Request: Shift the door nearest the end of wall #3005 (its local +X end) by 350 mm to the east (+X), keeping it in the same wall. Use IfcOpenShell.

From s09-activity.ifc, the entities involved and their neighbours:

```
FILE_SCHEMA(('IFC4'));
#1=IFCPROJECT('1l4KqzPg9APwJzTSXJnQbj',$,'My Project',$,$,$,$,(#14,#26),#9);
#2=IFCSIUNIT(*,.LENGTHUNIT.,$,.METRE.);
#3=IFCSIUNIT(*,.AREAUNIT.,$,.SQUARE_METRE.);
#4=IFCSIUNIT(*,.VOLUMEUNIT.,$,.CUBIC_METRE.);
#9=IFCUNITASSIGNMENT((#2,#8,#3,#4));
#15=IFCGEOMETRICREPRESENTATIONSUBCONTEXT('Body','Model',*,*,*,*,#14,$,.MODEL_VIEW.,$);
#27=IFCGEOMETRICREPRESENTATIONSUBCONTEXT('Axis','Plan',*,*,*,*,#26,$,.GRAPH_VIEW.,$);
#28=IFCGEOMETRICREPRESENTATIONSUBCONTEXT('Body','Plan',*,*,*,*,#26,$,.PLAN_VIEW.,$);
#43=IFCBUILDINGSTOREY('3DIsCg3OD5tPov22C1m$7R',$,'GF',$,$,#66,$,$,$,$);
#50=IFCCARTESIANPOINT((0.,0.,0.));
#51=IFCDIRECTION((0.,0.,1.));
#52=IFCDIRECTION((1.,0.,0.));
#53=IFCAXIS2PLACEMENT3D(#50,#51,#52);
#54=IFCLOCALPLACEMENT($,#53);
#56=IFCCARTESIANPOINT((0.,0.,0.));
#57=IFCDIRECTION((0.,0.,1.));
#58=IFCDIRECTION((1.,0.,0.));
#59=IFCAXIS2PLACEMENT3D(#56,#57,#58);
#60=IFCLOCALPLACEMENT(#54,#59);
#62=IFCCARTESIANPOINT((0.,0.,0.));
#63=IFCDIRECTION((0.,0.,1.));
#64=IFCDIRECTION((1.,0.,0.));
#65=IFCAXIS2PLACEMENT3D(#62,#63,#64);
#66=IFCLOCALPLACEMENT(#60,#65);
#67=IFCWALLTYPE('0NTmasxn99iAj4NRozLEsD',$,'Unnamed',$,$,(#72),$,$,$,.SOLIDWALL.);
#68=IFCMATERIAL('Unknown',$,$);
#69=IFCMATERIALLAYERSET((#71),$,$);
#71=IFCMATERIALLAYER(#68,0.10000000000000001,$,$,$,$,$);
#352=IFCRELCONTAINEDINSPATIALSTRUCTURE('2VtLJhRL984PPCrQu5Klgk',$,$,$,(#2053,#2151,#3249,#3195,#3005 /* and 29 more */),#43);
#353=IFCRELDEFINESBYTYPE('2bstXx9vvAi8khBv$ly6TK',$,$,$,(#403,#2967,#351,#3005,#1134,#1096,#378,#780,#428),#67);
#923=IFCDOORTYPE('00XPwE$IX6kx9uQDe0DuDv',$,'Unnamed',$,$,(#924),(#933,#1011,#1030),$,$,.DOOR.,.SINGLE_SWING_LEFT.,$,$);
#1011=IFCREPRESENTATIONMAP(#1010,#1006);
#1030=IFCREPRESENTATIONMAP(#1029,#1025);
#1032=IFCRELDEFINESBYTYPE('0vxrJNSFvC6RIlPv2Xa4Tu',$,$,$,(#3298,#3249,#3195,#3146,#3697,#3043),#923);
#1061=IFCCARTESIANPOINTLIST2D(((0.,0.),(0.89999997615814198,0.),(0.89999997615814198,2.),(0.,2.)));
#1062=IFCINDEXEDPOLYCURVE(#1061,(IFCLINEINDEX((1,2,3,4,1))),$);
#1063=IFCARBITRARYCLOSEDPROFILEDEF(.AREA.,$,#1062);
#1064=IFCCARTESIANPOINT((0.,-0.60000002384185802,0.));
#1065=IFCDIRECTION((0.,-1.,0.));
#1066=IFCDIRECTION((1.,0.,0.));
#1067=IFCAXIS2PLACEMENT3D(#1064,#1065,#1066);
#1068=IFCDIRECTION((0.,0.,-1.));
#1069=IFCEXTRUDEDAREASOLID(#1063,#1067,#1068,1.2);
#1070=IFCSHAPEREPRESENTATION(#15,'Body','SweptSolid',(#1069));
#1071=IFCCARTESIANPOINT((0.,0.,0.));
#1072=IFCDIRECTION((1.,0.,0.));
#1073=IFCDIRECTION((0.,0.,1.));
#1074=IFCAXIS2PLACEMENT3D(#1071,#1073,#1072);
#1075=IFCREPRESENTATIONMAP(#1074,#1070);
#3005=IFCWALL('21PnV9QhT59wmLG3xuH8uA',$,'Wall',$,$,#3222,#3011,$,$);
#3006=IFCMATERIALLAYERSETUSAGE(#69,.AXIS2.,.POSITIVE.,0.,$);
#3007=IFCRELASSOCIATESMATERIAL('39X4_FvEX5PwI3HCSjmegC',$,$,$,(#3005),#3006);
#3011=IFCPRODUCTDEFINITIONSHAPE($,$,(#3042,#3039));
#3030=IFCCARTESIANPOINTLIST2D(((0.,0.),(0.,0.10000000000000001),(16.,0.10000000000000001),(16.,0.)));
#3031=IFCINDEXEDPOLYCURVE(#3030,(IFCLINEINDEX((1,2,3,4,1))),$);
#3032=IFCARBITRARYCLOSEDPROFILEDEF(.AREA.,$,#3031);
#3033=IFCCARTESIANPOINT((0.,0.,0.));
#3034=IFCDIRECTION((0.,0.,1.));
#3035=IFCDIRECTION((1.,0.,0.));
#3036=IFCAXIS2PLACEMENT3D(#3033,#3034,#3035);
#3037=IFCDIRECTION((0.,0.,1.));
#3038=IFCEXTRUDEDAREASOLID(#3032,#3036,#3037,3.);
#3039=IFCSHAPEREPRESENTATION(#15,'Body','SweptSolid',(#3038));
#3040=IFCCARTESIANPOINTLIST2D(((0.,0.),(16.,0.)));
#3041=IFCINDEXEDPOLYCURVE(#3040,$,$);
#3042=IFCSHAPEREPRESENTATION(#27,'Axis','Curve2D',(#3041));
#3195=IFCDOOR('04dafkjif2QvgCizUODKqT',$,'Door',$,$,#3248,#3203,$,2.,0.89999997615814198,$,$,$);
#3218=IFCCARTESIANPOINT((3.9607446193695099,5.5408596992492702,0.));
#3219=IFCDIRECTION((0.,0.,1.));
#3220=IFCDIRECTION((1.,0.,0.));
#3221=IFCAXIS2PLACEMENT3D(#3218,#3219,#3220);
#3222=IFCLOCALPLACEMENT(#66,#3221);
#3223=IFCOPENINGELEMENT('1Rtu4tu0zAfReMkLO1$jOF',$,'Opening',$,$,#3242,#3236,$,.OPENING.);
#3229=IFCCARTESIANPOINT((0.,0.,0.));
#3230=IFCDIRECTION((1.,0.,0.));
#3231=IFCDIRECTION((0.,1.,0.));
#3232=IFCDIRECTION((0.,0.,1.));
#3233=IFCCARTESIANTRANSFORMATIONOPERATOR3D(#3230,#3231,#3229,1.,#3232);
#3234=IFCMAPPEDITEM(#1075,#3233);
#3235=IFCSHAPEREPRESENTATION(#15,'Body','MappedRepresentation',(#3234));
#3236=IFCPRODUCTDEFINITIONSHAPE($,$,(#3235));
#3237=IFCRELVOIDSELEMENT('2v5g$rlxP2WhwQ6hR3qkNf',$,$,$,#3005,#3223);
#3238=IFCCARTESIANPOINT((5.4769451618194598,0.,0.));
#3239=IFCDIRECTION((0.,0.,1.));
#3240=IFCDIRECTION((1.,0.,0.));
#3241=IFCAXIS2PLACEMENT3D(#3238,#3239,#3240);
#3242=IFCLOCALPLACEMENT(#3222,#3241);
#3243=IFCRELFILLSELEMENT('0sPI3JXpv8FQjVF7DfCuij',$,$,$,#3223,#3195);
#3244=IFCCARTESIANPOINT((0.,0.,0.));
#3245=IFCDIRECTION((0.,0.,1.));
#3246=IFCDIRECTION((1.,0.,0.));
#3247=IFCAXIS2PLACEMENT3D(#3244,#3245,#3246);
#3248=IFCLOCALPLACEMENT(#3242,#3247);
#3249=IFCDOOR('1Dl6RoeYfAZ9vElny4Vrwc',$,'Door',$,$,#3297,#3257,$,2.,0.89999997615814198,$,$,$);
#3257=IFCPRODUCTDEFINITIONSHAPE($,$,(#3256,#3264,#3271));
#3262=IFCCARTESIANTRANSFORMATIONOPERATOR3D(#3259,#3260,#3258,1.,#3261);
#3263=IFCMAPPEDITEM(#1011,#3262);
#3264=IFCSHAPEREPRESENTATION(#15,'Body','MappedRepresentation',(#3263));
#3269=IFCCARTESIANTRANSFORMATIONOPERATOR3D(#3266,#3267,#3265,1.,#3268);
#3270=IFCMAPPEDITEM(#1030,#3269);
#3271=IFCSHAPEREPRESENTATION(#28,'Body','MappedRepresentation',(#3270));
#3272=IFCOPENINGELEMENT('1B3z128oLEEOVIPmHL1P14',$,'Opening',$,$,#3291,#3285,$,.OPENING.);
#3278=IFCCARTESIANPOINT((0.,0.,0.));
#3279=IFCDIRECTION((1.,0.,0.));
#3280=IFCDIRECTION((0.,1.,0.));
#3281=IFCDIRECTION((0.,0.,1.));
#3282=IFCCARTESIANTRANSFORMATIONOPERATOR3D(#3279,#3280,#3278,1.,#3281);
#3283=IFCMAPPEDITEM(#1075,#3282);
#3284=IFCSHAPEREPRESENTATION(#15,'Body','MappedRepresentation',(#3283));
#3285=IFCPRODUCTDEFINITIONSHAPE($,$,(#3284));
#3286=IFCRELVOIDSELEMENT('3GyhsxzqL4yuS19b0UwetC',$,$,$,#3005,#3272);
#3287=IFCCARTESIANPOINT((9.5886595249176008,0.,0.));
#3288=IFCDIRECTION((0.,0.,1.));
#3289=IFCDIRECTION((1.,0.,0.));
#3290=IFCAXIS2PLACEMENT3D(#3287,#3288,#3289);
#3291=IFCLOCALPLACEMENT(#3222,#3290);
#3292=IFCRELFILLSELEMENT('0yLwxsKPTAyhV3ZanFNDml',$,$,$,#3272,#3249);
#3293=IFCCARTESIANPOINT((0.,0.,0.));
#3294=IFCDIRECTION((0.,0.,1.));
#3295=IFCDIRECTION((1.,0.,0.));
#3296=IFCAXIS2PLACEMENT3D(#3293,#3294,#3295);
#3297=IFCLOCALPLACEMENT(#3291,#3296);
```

```python
import ifcopenshell
import ifcopenshell.api.geometry
import ifcopenshell.util.placement
import ifcopenshell.util.unit

model = ifcopenshell.open("s09-activity.ifc")
unit_scale = ifcopenshell.util.unit.calculate_unit_scale(model)

door = model.by_guid("1Dl6RoeYfAZ9vElny4Vrwc")
opening = door.FillsVoids[0].RelatingOpeningElement
wall = opening.VoidsElements[0].RelatingBuildingElement

wall_matrix = ifcopenshell.util.placement.get_local_placement(wall.ObjectPlacement)
shift = wall_matrix[:3, 0] * 0.35 / unit_scale
before = ifcopenshell.util.placement.get_local_placement(door.ObjectPlacement)[:3, 3].copy()

# The door is placed relative to its opening, so it follows when the opening moves.
matrix = ifcopenshell.util.placement.get_local_placement(opening.ObjectPlacement)
matrix[:3, 3] += shift
ifcopenshell.api.geometry.edit_object_placement(
    model, product=opening, matrix=matrix, is_si=False, should_transform_children=True
)

after = ifcopenshell.util.placement.get_local_placement(door.ObjectPlacement)[:3, 3]
print("door moved by", (after - before).round(3) + 0.0)

model.write("s09-activity_v2.ifc")
```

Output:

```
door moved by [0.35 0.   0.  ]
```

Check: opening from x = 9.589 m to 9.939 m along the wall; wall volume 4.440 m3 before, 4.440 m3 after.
